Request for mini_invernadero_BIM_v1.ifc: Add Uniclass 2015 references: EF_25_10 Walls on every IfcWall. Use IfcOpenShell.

First a look at what the model holds.

```python
import ifcopenshell

model = ifcopenshell.open("mini_invernadero_BIM_v1.ifc")
print(model.schema)
print("classifications:", [c.Name for c in model.by_type("IfcClassification")])
for ifc_class in ("IfcDoor", "IfcRoof", "IfcStair", "IfcWall", "IfcWindow"):
    print(ifc_class, len(model.by_type(ifc_class)))
```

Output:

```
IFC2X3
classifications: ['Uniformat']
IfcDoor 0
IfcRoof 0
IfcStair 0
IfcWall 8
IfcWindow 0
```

```python
import ifcopenshell
import ifcopenshell.api.classification

model = ifcopenshell.open("mini_invernadero_BIM_v1.ifc")

# IFC2X3 requires Source and Edition and has no link from the project to the system.
system = model.create_entity("IfcClassification", Source="NBS", Edition="2015", Name="Uniclass 2015")

codes = {
    "IfcWall": ("EF_25_10", "Walls"),
}
for ifc_class, (code, name) in codes.items():
    products = model.by_type(ifc_class)
    ifcopenshell.api.classification.add_reference(
        model, products=products, classification=system, identification=code, name=name
    )
    print(code, len(products))

model.write("mini_invernadero_BIM_v1-out.ifc")
```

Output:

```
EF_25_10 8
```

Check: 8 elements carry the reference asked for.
